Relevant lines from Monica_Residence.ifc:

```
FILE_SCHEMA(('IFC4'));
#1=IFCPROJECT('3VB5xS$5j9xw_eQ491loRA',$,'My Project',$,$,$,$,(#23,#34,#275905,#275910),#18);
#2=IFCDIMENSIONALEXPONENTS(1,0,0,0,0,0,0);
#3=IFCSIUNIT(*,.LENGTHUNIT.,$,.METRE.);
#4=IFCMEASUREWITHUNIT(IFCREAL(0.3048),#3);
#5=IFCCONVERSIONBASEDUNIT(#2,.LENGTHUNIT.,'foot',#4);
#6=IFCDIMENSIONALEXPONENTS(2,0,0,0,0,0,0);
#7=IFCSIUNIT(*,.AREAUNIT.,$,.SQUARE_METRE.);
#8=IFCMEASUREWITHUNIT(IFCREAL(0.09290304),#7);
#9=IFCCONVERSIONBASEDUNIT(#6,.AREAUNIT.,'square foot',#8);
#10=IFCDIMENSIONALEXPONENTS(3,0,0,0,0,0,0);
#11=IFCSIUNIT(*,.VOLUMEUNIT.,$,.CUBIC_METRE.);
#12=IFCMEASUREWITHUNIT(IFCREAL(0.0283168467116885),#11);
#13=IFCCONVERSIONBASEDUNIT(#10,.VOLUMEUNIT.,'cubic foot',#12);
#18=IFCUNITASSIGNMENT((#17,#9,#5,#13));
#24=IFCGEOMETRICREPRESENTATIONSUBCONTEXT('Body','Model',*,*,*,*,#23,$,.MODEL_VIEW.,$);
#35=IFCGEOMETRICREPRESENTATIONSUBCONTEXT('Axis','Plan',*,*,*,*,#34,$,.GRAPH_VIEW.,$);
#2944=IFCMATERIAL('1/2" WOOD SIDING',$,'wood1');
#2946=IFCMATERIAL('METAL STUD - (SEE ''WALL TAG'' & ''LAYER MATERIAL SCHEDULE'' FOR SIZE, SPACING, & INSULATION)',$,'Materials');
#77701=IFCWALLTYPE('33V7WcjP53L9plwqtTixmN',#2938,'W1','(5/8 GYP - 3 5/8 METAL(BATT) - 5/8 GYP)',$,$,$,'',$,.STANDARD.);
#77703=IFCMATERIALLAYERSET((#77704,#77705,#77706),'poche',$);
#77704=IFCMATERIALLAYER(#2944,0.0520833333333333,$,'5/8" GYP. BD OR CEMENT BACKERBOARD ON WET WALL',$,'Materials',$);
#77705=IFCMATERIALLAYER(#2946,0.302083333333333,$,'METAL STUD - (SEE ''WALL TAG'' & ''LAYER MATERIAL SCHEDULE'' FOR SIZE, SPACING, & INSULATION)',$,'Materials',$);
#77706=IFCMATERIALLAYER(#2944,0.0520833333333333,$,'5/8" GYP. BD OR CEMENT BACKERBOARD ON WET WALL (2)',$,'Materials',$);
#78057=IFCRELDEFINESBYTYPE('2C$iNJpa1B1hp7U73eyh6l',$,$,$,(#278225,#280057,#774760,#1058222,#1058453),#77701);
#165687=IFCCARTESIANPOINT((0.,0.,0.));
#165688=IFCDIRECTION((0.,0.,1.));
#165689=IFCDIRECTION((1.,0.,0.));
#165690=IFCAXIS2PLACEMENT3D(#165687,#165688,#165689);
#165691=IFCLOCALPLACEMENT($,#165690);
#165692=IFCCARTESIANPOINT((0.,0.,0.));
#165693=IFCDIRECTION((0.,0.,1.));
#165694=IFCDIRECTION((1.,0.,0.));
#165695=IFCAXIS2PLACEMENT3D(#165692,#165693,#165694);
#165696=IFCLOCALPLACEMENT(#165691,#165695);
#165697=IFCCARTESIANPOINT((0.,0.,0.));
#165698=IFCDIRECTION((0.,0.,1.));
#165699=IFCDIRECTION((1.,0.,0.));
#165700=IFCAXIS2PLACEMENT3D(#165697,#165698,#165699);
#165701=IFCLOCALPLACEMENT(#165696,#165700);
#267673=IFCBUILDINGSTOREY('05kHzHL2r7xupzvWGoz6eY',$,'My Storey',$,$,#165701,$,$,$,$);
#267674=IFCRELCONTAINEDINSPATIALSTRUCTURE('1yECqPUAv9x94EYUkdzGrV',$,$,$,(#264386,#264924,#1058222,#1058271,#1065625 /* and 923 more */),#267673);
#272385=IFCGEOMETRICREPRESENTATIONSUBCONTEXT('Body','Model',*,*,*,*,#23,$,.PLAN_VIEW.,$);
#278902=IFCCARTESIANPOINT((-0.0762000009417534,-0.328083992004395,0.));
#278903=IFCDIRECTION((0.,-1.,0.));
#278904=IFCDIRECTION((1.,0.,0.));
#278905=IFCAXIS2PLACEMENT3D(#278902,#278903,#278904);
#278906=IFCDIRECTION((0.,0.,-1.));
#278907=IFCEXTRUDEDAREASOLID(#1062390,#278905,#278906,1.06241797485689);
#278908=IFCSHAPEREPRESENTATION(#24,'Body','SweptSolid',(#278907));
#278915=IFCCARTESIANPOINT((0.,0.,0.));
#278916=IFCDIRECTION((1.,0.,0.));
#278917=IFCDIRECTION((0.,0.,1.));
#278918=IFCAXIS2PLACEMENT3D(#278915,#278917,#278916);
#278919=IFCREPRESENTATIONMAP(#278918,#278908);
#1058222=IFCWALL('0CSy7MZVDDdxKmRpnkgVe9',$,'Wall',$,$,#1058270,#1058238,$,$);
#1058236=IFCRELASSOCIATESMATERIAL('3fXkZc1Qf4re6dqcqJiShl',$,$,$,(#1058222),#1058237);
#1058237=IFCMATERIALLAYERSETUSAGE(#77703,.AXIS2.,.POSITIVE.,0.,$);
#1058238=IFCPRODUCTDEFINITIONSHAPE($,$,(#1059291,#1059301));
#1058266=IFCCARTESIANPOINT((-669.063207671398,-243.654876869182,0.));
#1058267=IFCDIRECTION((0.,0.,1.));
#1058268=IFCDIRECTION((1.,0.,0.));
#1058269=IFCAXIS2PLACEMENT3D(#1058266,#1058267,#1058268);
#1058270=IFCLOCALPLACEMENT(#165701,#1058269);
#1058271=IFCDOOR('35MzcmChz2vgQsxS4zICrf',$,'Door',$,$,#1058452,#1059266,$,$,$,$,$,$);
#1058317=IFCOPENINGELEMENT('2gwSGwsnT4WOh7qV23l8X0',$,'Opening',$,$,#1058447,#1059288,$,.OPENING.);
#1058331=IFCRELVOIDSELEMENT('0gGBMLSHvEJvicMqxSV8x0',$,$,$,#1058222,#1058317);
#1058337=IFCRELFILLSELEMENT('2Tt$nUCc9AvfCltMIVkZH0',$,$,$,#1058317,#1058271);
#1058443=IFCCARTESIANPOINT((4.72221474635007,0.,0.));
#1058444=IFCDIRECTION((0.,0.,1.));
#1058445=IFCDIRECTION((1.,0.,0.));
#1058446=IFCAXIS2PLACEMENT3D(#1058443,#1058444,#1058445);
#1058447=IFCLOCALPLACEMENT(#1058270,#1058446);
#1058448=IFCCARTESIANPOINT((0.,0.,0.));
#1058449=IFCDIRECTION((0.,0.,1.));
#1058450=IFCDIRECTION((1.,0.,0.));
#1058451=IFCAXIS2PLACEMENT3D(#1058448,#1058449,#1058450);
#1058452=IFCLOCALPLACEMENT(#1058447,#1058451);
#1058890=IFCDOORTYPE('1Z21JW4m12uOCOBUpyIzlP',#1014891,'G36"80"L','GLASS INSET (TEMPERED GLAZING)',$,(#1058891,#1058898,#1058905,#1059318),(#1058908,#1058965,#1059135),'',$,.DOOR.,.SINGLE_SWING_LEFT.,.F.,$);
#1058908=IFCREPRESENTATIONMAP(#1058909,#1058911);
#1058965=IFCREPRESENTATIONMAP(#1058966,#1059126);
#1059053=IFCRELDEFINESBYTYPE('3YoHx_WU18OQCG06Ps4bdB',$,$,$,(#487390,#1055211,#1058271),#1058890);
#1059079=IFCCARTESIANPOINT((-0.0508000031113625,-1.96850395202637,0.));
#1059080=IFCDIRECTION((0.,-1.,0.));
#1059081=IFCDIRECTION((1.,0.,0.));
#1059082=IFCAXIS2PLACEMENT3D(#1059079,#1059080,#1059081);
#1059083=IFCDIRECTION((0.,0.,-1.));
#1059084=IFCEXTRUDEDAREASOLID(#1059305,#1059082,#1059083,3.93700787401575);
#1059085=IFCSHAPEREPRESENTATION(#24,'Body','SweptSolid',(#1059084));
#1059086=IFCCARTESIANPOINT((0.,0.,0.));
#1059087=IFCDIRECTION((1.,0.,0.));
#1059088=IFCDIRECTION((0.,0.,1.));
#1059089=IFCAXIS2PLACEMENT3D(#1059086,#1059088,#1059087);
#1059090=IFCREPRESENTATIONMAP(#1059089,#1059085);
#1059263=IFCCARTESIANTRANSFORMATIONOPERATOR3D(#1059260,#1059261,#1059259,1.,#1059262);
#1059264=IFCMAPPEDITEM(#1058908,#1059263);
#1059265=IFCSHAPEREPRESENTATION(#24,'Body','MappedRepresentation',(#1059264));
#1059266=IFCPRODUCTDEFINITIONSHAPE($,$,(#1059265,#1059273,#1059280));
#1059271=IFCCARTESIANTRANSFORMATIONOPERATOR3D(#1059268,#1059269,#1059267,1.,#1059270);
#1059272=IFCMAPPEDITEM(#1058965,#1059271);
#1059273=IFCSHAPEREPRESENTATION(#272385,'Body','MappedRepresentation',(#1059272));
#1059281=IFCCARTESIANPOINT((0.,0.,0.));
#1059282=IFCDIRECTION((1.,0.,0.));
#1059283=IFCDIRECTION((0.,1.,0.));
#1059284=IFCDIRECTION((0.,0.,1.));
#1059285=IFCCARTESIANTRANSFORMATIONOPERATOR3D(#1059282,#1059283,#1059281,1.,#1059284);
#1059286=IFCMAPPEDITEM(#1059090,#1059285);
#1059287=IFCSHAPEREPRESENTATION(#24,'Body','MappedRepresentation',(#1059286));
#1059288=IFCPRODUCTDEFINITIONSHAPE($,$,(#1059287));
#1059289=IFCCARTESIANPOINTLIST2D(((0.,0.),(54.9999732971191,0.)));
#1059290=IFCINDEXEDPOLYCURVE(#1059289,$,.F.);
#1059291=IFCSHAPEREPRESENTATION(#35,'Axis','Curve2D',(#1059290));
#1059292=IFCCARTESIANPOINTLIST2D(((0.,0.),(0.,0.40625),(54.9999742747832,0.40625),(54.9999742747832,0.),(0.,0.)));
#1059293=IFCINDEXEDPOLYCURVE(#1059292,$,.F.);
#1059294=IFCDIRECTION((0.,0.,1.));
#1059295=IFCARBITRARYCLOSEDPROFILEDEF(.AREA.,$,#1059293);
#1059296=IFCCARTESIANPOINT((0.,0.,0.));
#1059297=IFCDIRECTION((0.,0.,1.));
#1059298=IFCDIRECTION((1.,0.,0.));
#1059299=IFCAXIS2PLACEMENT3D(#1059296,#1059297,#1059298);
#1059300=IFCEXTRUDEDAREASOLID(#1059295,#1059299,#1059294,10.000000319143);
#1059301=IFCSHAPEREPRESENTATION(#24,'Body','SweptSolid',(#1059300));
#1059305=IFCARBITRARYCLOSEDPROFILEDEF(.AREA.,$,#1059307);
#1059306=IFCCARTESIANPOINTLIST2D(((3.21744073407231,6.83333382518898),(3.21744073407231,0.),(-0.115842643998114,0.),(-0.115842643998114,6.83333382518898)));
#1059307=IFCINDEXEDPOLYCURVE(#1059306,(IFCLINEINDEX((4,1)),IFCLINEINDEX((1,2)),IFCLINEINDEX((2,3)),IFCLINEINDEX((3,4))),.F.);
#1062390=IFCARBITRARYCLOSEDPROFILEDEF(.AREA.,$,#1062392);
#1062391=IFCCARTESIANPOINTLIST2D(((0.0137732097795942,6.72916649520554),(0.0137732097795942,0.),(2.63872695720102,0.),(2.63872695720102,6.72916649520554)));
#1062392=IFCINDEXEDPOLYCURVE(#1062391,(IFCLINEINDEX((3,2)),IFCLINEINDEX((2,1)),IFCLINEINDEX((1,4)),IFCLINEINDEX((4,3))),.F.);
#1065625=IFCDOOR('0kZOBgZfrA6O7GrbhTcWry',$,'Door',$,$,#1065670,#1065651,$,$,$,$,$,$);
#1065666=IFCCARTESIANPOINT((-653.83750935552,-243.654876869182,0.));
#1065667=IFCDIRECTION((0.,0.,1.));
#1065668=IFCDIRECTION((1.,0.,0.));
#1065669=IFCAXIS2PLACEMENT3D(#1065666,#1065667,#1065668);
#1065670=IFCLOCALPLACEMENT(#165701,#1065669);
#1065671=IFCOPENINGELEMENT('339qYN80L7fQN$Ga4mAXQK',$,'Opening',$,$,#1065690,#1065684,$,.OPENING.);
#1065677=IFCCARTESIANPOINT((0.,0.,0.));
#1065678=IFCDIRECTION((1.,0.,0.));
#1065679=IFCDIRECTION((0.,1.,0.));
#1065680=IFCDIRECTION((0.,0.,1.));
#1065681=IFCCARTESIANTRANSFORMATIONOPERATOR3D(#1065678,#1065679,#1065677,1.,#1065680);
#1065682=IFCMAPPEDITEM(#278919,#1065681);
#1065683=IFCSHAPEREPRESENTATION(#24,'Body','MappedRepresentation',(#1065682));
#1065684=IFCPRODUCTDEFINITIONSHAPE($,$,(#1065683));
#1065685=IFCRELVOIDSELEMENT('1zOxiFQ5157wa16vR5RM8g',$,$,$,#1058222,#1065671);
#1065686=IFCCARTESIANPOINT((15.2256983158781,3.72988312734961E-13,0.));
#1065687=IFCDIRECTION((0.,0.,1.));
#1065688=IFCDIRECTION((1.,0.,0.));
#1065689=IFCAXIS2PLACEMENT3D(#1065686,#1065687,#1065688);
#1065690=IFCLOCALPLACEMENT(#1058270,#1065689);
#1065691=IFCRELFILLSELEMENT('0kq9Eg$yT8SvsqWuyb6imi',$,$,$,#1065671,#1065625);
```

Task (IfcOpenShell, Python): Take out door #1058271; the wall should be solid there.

```python
import ifcopenshell
import ifcopenshell.api.feature
import ifcopenshell.api.root
import ifcopenshell.geom
import ifcopenshell.util.shape

model = ifcopenshell.open("Monica_Residence.ifc")
settings = ifcopenshell.geom.settings()


def volume(element):
    """Net volume in cubic metres, openings subtracted."""
    shape = ifcopenshell.geom.create_shape(settings, element)
    return ifcopenshell.util.shape.get_volume(shape.geometry)


door = model.by_guid("35MzcmChz2vgQsxS4zICrf")
opening = door.FillsVoids[0].RelatingOpeningElement
wall = opening.VoidsElements[0].RelatingBuildingElement
before = volume(wall)

ifcopenshell.api.root.remove_product(model, product=door)
ifcopenshell.api.feature.remove_feature(model, feature=opening)

after = volume(wall)

print(f"wall volume {before:.3f} -> {after:.3f} m3")

model.write("Monica_Residence_edited.ifc")
```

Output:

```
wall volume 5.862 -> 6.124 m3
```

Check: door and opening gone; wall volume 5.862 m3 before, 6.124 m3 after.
